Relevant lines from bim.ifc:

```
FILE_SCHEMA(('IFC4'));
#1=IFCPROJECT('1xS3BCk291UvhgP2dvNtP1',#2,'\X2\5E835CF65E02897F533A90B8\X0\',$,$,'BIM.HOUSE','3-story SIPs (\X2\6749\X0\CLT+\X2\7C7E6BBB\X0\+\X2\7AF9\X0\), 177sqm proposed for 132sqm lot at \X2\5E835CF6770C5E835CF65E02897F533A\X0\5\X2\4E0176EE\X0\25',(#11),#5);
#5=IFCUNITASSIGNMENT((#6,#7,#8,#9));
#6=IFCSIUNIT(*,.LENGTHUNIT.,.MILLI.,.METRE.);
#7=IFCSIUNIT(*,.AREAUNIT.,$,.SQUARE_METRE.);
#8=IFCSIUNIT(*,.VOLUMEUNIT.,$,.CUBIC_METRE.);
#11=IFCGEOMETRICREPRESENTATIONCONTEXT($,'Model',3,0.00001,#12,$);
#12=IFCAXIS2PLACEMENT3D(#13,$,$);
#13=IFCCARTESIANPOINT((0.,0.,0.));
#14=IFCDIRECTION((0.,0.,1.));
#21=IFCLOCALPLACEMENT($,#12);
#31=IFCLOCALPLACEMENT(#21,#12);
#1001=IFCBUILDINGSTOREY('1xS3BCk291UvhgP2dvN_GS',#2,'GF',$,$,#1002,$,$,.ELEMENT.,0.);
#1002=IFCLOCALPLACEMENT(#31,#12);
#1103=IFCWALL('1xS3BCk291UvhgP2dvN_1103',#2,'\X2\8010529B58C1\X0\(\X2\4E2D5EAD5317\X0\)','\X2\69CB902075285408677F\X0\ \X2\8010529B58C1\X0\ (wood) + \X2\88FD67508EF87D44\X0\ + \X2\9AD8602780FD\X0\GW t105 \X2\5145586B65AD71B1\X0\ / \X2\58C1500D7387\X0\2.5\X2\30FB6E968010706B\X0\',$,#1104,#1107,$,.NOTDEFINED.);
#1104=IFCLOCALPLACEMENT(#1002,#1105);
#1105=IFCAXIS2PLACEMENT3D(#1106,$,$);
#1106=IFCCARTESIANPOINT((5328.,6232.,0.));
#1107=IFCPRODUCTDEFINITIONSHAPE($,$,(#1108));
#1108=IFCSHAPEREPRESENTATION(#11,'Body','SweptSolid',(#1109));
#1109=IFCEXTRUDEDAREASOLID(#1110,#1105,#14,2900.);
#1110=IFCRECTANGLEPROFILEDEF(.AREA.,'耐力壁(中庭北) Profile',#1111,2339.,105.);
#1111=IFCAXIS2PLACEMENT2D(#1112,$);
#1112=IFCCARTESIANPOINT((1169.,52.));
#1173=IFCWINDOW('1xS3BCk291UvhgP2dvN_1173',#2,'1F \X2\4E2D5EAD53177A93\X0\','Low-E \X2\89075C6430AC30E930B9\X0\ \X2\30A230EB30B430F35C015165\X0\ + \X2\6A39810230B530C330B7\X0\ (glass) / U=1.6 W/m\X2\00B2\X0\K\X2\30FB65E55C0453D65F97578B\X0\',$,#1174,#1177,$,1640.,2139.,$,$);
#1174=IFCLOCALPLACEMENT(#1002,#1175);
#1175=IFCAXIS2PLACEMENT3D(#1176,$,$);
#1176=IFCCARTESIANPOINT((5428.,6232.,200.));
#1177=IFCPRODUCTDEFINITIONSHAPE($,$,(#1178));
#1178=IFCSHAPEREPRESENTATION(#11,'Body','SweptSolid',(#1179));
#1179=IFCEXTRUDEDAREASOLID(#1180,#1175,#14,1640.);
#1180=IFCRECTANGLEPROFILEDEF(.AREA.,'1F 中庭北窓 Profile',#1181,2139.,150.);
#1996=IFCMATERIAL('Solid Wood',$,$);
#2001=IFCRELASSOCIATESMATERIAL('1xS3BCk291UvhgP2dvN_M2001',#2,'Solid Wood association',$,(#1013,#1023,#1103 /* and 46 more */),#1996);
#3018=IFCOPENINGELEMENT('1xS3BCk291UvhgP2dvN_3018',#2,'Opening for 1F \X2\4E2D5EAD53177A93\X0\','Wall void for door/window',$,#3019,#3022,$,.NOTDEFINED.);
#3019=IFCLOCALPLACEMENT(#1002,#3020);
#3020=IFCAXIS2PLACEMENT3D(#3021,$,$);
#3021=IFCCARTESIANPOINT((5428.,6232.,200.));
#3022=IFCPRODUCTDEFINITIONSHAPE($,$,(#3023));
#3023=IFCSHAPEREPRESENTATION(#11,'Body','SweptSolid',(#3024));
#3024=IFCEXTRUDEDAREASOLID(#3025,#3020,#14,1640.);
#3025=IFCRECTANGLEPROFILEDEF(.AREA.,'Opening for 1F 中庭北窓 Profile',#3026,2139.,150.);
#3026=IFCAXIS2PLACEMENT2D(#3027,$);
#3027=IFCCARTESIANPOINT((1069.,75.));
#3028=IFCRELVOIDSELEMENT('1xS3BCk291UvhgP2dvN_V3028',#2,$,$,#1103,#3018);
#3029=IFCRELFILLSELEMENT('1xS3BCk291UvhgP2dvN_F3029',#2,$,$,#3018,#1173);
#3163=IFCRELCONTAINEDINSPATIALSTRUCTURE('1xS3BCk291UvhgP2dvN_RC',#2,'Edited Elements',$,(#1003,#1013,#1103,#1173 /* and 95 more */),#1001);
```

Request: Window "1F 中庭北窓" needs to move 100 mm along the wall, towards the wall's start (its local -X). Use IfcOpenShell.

```python
import ifcopenshell
import ifcopenshell.api.geometry
import ifcopenshell.util.placement
import ifcopenshell.util.unit

model = ifcopenshell.open("bim.ifc")
unit_scale = ifcopenshell.util.unit.calculate_unit_scale(model)

window = model.by_guid("1xS3BCk291UvhgP2dvN_1173")
opening = window.FillsVoids[0].RelatingOpeningElement
wall = opening.VoidsElements[0].RelatingBuildingElement

wall_matrix = ifcopenshell.util.placement.get_local_placement(wall.ObjectPlacement)
shift = wall_matrix[:3, 0] * -0.1 / unit_scale
before = ifcopenshell.util.placement.get_local_placement(window.ObjectPlacement)[:3, 3].copy()

# The window is not placed relative to its opening, so move both.
for product in (opening, window):
    matrix = ifcopenshell.util.placement.get_local_placement(product.ObjectPlacement)
    matrix[:3, 3] += shift
    ifcopenshell.api.geometry.edit_object_placement(model, product=product, matrix=matrix, is_si=False)

after = ifcopenshell.util.placement.get_local_placement(window.ObjectPlacement)[:3, 3]
print("window moved by", (after - before).round(3) + 0.0)

model.write("bim_v2.ifc")
```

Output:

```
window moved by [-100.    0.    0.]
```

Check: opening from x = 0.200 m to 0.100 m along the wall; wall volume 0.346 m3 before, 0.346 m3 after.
